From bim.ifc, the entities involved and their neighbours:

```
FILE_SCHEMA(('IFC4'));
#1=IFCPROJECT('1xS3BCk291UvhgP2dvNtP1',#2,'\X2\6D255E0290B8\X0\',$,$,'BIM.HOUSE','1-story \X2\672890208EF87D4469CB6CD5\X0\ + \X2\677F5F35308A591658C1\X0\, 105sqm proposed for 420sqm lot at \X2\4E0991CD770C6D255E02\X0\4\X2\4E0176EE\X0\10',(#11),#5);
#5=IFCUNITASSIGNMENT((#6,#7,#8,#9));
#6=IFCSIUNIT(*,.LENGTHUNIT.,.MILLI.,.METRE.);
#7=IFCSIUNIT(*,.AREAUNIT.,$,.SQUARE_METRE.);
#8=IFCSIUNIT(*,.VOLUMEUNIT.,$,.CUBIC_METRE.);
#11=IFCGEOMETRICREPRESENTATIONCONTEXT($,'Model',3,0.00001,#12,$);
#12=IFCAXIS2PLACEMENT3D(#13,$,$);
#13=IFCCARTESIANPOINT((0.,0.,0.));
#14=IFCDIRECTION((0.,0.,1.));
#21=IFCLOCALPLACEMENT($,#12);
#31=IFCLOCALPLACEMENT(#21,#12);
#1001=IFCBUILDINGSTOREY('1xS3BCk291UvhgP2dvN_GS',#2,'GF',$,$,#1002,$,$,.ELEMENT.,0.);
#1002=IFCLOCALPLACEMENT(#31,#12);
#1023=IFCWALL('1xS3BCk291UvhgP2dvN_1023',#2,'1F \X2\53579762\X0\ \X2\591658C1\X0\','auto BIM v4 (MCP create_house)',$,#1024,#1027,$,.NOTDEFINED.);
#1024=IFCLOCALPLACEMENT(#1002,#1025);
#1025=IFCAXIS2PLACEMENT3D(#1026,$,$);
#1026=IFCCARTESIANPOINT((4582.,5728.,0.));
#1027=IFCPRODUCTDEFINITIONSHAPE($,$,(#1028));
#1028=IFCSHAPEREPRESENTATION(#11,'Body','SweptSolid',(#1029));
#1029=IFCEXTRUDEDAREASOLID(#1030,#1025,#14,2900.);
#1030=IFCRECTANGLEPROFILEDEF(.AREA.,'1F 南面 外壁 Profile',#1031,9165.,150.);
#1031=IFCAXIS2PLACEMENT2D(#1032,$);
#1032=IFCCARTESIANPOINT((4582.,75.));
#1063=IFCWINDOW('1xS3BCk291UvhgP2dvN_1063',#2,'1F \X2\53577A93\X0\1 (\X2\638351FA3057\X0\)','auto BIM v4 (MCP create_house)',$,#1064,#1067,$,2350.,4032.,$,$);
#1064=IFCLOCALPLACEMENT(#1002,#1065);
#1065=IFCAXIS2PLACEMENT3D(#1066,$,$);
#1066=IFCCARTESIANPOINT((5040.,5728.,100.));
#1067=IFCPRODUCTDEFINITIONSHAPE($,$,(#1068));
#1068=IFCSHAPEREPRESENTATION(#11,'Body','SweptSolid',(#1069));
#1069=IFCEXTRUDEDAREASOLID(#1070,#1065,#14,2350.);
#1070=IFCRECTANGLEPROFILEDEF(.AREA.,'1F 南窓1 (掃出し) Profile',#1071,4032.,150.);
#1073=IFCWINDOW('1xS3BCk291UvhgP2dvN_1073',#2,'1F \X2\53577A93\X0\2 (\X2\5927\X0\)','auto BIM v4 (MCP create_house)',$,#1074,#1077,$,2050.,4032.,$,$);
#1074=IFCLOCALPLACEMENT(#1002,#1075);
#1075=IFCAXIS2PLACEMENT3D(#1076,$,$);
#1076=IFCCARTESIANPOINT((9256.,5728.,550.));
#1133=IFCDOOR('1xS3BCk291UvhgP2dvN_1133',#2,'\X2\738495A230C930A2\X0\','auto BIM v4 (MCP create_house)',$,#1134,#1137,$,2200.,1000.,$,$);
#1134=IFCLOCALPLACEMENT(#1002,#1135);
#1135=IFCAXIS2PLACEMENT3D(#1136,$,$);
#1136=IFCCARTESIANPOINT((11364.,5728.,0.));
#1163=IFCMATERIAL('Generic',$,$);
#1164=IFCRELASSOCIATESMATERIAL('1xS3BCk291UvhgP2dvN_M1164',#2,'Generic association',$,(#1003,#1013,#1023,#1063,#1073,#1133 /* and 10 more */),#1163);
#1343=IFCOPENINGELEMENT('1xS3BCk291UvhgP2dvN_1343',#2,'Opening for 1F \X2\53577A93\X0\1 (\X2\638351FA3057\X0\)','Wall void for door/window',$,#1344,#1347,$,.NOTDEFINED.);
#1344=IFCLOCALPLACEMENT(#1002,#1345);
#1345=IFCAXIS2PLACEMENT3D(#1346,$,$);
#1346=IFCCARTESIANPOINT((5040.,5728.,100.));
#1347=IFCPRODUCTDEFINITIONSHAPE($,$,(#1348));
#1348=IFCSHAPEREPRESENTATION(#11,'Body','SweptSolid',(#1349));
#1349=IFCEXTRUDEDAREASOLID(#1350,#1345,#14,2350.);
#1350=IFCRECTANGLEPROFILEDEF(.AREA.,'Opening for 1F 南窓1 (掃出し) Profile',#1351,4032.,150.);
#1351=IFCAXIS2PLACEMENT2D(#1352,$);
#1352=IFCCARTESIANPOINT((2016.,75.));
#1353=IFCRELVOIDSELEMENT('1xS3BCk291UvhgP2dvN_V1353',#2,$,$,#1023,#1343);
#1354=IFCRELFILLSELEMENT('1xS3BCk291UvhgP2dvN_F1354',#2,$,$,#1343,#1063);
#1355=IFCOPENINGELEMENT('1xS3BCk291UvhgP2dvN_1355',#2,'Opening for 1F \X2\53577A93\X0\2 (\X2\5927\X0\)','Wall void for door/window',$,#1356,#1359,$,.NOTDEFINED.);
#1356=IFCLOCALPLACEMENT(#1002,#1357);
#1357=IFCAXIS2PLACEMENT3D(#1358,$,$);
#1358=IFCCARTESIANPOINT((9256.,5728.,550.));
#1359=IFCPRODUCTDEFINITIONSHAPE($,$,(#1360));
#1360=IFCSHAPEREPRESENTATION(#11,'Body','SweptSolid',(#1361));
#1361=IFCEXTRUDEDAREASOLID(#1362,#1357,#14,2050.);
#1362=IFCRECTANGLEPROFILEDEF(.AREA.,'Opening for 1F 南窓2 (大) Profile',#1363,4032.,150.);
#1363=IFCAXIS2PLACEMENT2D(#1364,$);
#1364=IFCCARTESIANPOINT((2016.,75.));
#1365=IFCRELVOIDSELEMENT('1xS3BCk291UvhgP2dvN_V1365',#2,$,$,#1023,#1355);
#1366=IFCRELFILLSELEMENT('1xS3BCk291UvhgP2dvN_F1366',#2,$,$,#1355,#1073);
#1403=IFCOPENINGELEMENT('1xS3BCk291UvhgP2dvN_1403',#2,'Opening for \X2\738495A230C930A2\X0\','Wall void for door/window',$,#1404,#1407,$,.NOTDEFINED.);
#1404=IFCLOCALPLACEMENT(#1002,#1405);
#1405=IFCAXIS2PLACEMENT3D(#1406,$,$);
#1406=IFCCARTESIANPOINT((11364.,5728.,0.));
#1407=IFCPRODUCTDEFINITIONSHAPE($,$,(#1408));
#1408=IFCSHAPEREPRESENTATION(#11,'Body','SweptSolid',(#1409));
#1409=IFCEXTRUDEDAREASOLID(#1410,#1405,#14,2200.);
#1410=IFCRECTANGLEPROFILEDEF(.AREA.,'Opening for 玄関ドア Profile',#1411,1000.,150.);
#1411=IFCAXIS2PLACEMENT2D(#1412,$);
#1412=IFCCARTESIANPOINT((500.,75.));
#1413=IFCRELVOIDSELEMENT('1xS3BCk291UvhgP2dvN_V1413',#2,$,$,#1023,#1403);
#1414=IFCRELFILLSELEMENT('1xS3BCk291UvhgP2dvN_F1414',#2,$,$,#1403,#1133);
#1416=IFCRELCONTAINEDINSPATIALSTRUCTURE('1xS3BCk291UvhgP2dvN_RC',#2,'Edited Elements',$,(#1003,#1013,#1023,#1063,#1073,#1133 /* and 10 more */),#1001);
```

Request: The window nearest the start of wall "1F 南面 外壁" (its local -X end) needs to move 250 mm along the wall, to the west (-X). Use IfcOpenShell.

```python
import ifcopenshell
import ifcopenshell.api.geometry
import ifcopenshell.util.placement
import ifcopenshell.util.unit

model = ifcopenshell.open("bim.ifc")
unit_scale = ifcopenshell.util.unit.calculate_unit_scale(model)

window = model.by_guid("1xS3BCk291UvhgP2dvN_1063")
opening = window.FillsVoids[0].RelatingOpeningElement
wall = opening.VoidsElements[0].RelatingBuildingElement

wall_matrix = ifcopenshell.util.placement.get_local_placement(wall.ObjectPlacement)
shift = wall_matrix[:3, 0] * -0.25 / unit_scale
before = ifcopenshell.util.placement.get_local_placement(window.ObjectPlacement)[:3, 3].copy()

# The window is not placed relative to its opening, so move both.
for product in (opening, window):
    matrix = ifcopenshell.util.placement.get_local_placement(product.ObjectPlacement)
    matrix[:3, 3] += shift
    ifcopenshell.api.geometry.edit_object_placement(model, product=product, matrix=matrix, is_si=False)

after = ifcopenshell.util.placement.get_local_placement(window.ObjectPlacement)[:3, 3]
print("window moved by", (after - before).round(3) + 0.0)

model.write("bim_edited.ifc")
```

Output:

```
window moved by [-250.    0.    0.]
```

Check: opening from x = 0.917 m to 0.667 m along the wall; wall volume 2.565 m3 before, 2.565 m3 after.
